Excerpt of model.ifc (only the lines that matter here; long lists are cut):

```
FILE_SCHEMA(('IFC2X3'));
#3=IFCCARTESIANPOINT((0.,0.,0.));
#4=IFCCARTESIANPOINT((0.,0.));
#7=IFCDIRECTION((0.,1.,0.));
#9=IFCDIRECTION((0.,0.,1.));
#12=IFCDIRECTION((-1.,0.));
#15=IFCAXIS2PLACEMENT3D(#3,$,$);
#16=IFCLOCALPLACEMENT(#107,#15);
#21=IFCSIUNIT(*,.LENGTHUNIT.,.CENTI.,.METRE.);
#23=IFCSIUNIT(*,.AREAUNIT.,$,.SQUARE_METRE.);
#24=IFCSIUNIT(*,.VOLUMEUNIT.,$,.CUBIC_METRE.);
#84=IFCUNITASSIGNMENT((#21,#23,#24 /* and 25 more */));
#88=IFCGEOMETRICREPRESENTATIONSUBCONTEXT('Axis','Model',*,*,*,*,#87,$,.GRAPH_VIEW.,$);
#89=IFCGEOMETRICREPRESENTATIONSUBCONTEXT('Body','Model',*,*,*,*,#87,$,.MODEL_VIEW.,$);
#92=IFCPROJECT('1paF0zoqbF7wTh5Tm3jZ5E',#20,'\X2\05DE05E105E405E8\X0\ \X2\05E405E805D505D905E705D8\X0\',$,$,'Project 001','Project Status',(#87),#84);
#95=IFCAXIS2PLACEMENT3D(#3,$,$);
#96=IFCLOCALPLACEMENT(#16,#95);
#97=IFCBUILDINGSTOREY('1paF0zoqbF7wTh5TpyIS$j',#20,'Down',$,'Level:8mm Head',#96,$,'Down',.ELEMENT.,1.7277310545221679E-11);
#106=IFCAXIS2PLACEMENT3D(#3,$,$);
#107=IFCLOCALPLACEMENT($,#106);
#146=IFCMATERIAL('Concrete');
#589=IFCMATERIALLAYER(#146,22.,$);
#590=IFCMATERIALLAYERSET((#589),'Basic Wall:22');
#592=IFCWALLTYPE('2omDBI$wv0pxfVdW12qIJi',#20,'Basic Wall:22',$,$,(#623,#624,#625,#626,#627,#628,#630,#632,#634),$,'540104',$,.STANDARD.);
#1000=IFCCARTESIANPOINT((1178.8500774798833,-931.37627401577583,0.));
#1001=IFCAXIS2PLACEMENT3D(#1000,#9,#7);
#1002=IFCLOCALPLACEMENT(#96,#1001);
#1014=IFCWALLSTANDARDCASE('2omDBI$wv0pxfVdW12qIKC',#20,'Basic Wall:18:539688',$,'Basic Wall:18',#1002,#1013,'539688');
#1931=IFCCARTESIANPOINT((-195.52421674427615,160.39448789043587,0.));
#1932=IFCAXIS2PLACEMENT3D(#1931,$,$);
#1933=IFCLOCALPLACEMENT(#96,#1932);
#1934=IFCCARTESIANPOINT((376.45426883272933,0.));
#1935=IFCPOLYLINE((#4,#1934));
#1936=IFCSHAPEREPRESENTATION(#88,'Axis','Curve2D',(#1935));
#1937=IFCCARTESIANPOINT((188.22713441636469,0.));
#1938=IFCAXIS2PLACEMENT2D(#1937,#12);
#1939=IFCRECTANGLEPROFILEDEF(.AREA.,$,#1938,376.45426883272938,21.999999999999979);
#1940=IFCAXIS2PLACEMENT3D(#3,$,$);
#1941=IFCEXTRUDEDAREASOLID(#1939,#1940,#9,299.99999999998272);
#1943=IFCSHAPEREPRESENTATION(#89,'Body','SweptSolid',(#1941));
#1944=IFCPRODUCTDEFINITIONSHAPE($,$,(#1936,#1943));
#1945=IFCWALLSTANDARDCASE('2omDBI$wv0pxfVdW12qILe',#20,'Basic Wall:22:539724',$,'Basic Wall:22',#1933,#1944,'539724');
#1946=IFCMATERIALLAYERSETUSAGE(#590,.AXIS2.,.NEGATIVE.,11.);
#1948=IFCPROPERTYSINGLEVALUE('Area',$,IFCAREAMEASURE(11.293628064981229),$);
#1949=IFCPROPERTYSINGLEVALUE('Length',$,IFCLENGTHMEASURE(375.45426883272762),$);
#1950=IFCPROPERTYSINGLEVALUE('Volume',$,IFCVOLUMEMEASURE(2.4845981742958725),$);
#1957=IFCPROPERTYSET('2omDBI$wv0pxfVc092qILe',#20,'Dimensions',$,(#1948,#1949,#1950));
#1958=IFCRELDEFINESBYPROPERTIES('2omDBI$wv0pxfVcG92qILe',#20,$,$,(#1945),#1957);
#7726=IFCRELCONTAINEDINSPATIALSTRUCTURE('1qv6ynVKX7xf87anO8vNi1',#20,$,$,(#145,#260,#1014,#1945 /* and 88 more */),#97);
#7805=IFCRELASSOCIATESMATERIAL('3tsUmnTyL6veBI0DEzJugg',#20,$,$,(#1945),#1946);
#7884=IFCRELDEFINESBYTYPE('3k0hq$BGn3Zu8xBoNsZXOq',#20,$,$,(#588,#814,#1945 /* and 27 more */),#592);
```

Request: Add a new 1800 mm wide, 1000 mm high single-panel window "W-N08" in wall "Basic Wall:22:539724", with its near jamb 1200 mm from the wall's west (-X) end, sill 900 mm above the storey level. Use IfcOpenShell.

```python
import numpy as np
import ifcopenshell
import ifcopenshell.api.feature
import ifcopenshell.api.geometry
import ifcopenshell.api.pset
import ifcopenshell.api.root
import ifcopenshell.api.spatial
import ifcopenshell.api.type
import ifcopenshell.geom
import ifcopenshell.util.element
import ifcopenshell.util.placement
import ifcopenshell.util.representation
import ifcopenshell.util.shape
import ifcopenshell.util.unit

model = ifcopenshell.open("model.ifc")
unit_scale = ifcopenshell.util.unit.calculate_unit_scale(model)
area_scale = ifcopenshell.util.unit.calculate_unit_scale(model, "AREAUNIT")
volume_scale = ifcopenshell.util.unit.calculate_unit_scale(model, "VOLUMEUNIT")
settings = ifcopenshell.geom.settings()


def volume(element):
    """Net volume in cubic metres, openings subtracted."""
    shape = ifcopenshell.geom.create_shape(settings, element)
    return ifcopenshell.util.shape.get_volume(shape.geometry)


wall = model.by_id(1945)
storey = ifcopenshell.util.element.get_container(wall, ifc_class="IfcBuildingStorey")
context = ifcopenshell.util.representation.get_context(model, "Model", "Body", "MODEL_VIEW")
before = volume(wall)

width, height, from_end, sill = 1.8, 1, 1.2, 0.9  # metres

# The wall runs along its own X axis, and the end named is its -X end.
wall_shape = ifcopenshell.geom.create_shape(settings, wall)
x, y, z = ifcopenshell.util.shape.get_vertices(wall_shape.geometry).T
start = x.min() + from_end
face, thickness = float(y.min()), float(y.max() - y.min())
wall_matrix = ifcopenshell.util.placement.get_local_placement(wall.ObjectPlacement)
level = ifcopenshell.util.placement.get_local_placement(storey.ObjectPlacement)[2, 3]


def in_wall(x, y):
    """Placement at x, y metres in the wall's axes, at sill height."""
    matrix = wall_matrix.copy()
    matrix[:, 3] = wall_matrix @ np.array([x / unit_scale, y / unit_scale, 0.0, 1.0])
    matrix[2, 3] = level + sill / unit_scale
    return matrix


# Opening: a box that overshoots both wall faces by 50 mm.
opening = ifcopenshell.api.root.create_entity(model, ifc_class="IfcOpeningElement")
box = ifcopenshell.api.geometry.add_wall_representation(
    model, context=context, length=width, height=height, thickness=thickness + 0.1
)
ifcopenshell.api.geometry.assign_representation(model, product=opening, representation=box)
ifcopenshell.api.geometry.edit_object_placement(model, product=opening, matrix=in_wall(start, face - 0.05), is_si=False)
ifcopenshell.api.feature.add_feature(model, feature=opening, element=wall)

window = ifcopenshell.api.root.create_entity(model, ifc_class="IfcWindow", name="W-N08")
window.OverallWidth, window.OverallHeight = width / unit_scale, height / unit_scale
body = ifcopenshell.api.geometry.add_window_representation(
    model,
    context=context,
    overall_width=window.OverallWidth,
    overall_height=window.OverallHeight,
    partition_type="SINGLE_PANEL",
)
ifcopenshell.api.geometry.assign_representation(model, product=window, representation=body)
ifcopenshell.api.spatial.assign_container(model, products=[window], relating_structure=storey)
fills = ifcopenshell.api.feature.add_filling(model, opening=opening, element=window)
fills.OwnerHistory = window.OwnerHistory  # required in IFC2X3

# IFC2X3 keeps the operation on the window style.
style = ifcopenshell.api.root.create_entity(model, ifc_class="IfcWindowStyle", name="W-N08")
style.OperationType, style.ConstructionType = "SINGLE_PANEL", "NOTDEFINED"
style.ParameterTakesPrecedence = style.Sizeable = False
ifcopenshell.api.type.assign_type(model, related_objects=[window], relating_type=style)

# Centre the window in the wall's thickness.
ifcopenshell.api.geometry.edit_object_placement(model, product=window, matrix=in_wall(start, face), is_si=False)
window_shape = ifcopenshell.geom.create_shape(settings, window)
depth = ifcopenshell.util.shape.get_vertices(window_shape.geometry)[:, 1]
offset = face + thickness / 2 - (depth.min() + depth.max()) / 2
ifcopenshell.api.geometry.edit_object_placement(model, product=window, matrix=in_wall(start, offset), is_si=False)

after = volume(wall)

# Update the wall's stored quantities.
pset = model.by_id(ifcopenshell.util.element.get_pset(wall, "Dimensions", should_inherit=False)["id"])
ifcopenshell.api.pset.edit_pset(model, pset=pset, properties={
    "Area": model.create_entity("IfcAreaMeasure", after / thickness / area_scale),
    "Volume": model.create_entity("IfcVolumeMeasure", after / volume_scale),
})

print(f"wall volume {before:.3f} -> {after:.3f} m3")

model.write("model-out.ifc")
```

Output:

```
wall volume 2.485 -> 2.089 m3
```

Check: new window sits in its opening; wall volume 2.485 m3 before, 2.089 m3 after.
